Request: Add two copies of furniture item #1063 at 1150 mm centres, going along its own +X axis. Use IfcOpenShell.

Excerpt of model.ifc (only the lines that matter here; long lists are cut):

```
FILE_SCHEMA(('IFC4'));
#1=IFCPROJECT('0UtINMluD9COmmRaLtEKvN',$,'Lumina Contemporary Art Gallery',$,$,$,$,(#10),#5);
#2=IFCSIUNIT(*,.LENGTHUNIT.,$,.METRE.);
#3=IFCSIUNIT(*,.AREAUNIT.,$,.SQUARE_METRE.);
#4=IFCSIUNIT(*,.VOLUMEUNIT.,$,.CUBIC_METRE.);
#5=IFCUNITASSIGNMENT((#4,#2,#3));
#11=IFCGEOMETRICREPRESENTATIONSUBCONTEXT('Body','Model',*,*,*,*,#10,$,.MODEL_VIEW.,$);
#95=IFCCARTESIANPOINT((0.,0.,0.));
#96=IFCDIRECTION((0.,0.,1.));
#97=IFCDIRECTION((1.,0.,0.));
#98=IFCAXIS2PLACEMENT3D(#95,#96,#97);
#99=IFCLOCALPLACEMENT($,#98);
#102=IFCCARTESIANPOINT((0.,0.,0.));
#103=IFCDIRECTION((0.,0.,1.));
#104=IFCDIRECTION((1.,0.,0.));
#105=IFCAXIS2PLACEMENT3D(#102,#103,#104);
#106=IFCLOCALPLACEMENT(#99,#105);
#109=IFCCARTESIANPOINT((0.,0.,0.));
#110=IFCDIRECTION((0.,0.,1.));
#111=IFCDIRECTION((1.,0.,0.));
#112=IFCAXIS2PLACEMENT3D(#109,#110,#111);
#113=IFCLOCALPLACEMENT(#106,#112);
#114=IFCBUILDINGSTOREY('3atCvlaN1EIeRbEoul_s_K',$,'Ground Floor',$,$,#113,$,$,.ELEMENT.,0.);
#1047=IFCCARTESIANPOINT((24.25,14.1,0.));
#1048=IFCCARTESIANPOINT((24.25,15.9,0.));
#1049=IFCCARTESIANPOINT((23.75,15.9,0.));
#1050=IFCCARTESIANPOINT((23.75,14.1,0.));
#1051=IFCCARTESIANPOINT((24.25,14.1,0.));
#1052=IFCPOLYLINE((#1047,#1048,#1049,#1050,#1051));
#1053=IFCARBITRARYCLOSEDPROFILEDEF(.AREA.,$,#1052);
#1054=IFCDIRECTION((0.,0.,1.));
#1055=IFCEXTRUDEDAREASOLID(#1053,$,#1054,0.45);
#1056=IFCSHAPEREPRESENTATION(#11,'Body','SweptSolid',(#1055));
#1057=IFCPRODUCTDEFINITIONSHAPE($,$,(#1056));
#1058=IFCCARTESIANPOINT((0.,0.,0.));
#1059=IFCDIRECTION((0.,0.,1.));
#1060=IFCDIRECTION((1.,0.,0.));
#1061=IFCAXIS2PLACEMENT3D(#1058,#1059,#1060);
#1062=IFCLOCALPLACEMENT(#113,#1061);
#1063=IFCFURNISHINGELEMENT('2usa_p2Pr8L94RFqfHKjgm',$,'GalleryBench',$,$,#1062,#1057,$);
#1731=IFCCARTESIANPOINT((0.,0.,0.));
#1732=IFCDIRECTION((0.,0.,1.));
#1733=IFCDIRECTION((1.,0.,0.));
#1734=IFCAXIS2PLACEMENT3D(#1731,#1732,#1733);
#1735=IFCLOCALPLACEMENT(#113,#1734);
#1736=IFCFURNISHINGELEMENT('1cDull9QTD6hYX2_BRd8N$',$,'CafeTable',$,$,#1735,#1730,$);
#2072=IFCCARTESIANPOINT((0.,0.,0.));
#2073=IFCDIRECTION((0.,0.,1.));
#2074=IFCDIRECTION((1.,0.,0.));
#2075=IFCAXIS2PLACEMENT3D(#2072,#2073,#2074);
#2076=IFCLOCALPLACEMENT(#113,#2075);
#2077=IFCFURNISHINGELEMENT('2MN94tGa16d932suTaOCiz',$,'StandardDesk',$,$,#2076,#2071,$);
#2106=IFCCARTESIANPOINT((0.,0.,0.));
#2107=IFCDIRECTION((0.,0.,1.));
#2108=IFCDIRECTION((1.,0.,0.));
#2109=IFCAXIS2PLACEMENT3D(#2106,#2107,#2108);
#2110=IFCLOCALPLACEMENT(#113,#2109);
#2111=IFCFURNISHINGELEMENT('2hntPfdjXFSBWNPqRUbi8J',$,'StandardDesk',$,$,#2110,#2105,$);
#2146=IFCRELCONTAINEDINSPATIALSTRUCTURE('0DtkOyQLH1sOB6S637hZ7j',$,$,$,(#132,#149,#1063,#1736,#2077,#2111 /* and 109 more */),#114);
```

```python
import ifcopenshell
import ifcopenshell.api.geometry
import ifcopenshell.api.root
import ifcopenshell.util.element
import ifcopenshell.util.placement

model = ifcopenshell.open("model.ifc")

source = model.by_guid("2usa_p2Pr8L94RFqfHKjgm")
base = ifcopenshell.util.placement.get_local_placement(source.ObjectPlacement)
step = base[:3, 0] * 1.15

for i in range(1, 3):
    copy = ifcopenshell.api.root.copy_class(model, product=source)
    copy.Representation = ifcopenshell.util.element.copy_deep(
        model, source.Representation, exclude=["IfcGeometricRepresentationContext", "IfcRepresentationMap"]
    )
    matrix = base.copy()
    matrix[:3, 3] += i * step
    print("added at", matrix[:3, 3].round(3) + 0.0)
    ifcopenshell.api.geometry.edit_object_placement(model, product=copy, matrix=matrix, is_si=False)

model.write("model_updated.ifc")
```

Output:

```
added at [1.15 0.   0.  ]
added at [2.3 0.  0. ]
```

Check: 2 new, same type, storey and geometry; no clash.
